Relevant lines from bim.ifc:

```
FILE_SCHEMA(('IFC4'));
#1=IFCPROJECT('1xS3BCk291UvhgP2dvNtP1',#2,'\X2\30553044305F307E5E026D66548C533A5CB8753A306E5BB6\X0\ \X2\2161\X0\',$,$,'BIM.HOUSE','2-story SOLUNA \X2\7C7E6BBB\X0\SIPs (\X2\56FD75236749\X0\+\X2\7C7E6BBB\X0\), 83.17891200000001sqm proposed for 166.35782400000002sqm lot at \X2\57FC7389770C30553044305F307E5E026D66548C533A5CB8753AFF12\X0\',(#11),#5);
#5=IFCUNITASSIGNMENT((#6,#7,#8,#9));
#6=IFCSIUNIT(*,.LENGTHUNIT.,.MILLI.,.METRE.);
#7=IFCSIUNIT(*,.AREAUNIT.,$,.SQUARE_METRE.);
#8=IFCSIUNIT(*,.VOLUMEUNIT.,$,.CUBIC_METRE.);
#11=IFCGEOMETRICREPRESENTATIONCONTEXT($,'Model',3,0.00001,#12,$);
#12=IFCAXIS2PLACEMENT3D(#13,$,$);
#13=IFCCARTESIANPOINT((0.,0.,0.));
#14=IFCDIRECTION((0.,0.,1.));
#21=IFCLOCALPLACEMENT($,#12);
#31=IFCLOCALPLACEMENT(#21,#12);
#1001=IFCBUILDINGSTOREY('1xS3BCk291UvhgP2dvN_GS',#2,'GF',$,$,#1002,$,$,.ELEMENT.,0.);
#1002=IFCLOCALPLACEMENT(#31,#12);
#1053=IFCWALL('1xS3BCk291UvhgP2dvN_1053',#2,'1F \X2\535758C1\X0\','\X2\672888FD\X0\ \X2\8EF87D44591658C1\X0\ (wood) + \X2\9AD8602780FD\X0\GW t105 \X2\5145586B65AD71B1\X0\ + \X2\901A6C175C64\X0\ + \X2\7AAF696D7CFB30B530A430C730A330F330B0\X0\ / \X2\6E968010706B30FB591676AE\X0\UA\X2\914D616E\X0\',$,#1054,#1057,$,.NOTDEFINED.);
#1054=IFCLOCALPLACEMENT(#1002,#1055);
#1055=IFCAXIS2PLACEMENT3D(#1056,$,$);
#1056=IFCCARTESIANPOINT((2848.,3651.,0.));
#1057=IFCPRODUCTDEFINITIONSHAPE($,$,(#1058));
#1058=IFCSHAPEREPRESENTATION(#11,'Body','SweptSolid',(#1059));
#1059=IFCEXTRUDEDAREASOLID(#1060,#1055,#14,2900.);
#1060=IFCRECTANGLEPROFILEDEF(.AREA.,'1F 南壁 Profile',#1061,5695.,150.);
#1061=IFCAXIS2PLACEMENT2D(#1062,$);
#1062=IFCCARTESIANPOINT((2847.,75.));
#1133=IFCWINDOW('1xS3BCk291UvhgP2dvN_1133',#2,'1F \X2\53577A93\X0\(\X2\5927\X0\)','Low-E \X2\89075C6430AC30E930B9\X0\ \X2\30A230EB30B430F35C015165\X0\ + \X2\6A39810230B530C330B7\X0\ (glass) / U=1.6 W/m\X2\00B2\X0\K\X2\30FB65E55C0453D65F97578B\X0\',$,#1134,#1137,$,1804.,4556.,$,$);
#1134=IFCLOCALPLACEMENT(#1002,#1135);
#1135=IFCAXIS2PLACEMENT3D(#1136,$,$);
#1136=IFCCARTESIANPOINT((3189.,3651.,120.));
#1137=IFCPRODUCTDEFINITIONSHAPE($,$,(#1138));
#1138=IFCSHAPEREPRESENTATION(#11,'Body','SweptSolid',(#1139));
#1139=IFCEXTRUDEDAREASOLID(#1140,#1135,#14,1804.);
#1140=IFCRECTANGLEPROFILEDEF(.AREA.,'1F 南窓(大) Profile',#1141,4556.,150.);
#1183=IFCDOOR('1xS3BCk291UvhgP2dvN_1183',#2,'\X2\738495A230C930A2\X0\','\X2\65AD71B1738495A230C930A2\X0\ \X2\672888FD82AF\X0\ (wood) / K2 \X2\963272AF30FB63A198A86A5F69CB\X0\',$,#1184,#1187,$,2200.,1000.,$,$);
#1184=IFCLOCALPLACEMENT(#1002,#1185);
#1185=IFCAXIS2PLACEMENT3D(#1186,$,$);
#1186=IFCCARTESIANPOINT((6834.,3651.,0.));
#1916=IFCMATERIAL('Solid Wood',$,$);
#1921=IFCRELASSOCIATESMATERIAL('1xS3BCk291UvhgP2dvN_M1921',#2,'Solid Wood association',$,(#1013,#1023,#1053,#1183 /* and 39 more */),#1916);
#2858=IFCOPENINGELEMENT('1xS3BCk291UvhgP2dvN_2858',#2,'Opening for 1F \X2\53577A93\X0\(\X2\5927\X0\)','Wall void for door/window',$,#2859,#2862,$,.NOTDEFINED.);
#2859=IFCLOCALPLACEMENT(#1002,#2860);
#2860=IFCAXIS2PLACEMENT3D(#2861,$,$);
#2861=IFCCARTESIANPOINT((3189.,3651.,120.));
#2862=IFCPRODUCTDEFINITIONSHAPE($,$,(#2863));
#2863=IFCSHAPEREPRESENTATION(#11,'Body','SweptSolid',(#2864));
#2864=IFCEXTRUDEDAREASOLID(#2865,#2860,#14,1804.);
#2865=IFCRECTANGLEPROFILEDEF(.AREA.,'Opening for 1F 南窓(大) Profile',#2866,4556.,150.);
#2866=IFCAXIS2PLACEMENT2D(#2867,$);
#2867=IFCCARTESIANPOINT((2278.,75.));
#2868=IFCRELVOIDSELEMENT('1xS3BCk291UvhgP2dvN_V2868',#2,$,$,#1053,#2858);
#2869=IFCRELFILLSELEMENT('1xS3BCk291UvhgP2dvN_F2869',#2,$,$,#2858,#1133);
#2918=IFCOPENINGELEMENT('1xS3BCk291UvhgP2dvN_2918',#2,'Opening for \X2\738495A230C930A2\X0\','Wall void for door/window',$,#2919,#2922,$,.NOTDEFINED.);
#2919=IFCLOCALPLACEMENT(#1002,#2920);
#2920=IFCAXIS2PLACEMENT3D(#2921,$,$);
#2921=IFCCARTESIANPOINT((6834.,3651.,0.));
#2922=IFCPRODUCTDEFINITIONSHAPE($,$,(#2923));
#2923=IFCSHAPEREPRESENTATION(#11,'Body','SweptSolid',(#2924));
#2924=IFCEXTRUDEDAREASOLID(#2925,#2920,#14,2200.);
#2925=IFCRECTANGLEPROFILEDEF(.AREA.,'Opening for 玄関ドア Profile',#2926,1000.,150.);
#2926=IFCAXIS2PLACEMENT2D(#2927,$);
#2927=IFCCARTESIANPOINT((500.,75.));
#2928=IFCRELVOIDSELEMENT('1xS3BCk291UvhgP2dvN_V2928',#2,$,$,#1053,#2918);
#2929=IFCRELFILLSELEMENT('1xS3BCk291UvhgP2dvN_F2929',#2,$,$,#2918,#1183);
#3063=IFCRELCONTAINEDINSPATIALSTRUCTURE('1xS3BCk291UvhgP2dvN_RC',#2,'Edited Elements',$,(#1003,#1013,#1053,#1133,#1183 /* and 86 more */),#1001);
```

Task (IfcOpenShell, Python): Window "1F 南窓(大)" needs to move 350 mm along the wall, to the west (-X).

```python
import ifcopenshell
import ifcopenshell.api.geometry
import ifcopenshell.util.placement
import ifcopenshell.util.unit

model = ifcopenshell.open("bim.ifc")
unit_scale = ifcopenshell.util.unit.calculate_unit_scale(model)

window = model.by_guid("1xS3BCk291UvhgP2dvN_1133")
opening = window.FillsVoids[0].RelatingOpeningElement
wall = opening.VoidsElements[0].RelatingBuildingElement

wall_matrix = ifcopenshell.util.placement.get_local_placement(wall.ObjectPlacement)
shift = wall_matrix[:3, 0] * -0.35 / unit_scale
before = ifcopenshell.util.placement.get_local_placement(window.ObjectPlacement)[:3, 3].copy()

# The window is not placed relative to its opening, so move both.
for product in (opening, window):
    matrix = ifcopenshell.util.placement.get_local_placement(product.ObjectPlacement)
    matrix[:3, 3] += shift
    ifcopenshell.api.geometry.edit_object_placement(model, product=product, matrix=matrix, is_si=False)

after = ifcopenshell.util.placement.get_local_placement(window.ObjectPlacement)[:3, 3]
print("window moved by", (after - before).round(3) + 0.0)

model.write("bim_edited.ifc")
```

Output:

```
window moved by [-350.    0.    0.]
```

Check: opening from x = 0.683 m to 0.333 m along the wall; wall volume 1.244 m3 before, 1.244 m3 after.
